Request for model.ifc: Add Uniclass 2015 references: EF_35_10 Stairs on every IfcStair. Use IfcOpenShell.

First a look at what the model holds.

```python
import ifcopenshell

model = ifcopenshell.open("model.ifc")
print(model.schema)
print("classifications:", [c.Name for c in model.by_type("IfcClassification")])
for ifc_class in ("IfcDoor", "IfcRoof", "IfcStair", "IfcWall", "IfcWindow"):
    print(ifc_class, len(model.by_type(ifc_class)))
```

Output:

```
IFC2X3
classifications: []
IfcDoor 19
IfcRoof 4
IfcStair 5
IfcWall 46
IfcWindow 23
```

```python
import ifcopenshell
import ifcopenshell.api.classification

model = ifcopenshell.open("model.ifc")

# IFC2X3 requires Source and Edition and has no link from the project to the system.
system = model.create_entity("IfcClassification", Source="NBS", Edition="2015", Name="Uniclass 2015")

codes = {
    "IfcStair": ("EF_35_10", "Stairs"),
}
for ifc_class, (code, name) in codes.items():
    products = model.by_type(ifc_class)
    ifcopenshell.api.classification.add_reference(
        model, products=products, classification=system, identification=code, name=name
    )
    print(code, len(products))

model.write("model_updated.ifc")
```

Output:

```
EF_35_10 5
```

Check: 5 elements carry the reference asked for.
